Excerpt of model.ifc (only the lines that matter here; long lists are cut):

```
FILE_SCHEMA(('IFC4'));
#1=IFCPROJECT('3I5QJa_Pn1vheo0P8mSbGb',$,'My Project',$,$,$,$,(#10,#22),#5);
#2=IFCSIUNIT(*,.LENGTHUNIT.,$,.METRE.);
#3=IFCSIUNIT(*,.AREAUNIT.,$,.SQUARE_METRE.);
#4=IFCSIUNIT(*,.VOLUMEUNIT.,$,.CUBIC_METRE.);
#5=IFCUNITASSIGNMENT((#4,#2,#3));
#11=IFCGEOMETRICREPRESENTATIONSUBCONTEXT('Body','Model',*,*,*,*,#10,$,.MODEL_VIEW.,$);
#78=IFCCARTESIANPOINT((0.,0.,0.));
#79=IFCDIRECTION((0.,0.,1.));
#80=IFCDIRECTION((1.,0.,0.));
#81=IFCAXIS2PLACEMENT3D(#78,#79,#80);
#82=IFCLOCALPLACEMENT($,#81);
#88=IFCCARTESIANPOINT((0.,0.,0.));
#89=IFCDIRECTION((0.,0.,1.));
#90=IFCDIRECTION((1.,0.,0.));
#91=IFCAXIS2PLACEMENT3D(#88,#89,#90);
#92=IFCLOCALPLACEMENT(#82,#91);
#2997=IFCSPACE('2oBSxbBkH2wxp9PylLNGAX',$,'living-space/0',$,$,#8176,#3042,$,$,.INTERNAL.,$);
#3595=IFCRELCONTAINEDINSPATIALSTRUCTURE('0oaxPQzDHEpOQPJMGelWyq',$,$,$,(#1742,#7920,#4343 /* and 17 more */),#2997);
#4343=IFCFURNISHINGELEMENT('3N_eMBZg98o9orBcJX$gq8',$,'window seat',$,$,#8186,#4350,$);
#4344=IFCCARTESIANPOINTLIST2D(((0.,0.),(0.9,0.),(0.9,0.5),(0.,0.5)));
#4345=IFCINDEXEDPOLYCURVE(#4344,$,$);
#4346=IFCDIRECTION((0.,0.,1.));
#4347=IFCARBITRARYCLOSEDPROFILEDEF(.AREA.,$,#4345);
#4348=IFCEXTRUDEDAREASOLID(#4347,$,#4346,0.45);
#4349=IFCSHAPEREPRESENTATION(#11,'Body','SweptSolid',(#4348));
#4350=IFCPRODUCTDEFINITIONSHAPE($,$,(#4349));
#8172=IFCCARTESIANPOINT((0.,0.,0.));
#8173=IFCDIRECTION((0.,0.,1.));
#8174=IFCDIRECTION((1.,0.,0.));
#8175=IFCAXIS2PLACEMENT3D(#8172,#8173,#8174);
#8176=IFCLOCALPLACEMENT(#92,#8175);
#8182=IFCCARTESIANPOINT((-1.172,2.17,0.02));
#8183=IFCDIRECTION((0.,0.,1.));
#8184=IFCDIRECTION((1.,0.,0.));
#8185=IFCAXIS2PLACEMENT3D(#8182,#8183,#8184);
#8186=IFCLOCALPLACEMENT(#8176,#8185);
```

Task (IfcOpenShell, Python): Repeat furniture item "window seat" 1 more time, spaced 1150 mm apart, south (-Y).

```python
import numpy as np
import ifcopenshell
import ifcopenshell.api.geometry
import ifcopenshell.api.root
import ifcopenshell.util.element
import ifcopenshell.util.placement
import ifcopenshell.util.unit

model = ifcopenshell.open("model.ifc")
unit_scale = ifcopenshell.util.unit.calculate_unit_scale(model)

source = model.by_guid("3N_eMBZg98o9orBcJX$gq8")
base = ifcopenshell.util.placement.get_local_placement(source.ObjectPlacement)
step = np.array([0.0, -1.0, 0.0]) * 1.15 / unit_scale

for i in range(1, 2):
    copy = ifcopenshell.api.root.copy_class(model, product=source)
    copy.Representation = ifcopenshell.util.element.copy_deep(
        model, source.Representation, exclude=["IfcGeometricRepresentationContext", "IfcRepresentationMap"]
    )
    matrix = base.copy()
    matrix[:3, 3] += i * step
    print("added at", matrix[:3, 3].round(3) + 0.0)
    ifcopenshell.api.geometry.edit_object_placement(model, product=copy, matrix=matrix, is_si=False)

model.write("model_updated.ifc")
```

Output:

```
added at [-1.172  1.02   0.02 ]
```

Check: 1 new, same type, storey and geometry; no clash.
